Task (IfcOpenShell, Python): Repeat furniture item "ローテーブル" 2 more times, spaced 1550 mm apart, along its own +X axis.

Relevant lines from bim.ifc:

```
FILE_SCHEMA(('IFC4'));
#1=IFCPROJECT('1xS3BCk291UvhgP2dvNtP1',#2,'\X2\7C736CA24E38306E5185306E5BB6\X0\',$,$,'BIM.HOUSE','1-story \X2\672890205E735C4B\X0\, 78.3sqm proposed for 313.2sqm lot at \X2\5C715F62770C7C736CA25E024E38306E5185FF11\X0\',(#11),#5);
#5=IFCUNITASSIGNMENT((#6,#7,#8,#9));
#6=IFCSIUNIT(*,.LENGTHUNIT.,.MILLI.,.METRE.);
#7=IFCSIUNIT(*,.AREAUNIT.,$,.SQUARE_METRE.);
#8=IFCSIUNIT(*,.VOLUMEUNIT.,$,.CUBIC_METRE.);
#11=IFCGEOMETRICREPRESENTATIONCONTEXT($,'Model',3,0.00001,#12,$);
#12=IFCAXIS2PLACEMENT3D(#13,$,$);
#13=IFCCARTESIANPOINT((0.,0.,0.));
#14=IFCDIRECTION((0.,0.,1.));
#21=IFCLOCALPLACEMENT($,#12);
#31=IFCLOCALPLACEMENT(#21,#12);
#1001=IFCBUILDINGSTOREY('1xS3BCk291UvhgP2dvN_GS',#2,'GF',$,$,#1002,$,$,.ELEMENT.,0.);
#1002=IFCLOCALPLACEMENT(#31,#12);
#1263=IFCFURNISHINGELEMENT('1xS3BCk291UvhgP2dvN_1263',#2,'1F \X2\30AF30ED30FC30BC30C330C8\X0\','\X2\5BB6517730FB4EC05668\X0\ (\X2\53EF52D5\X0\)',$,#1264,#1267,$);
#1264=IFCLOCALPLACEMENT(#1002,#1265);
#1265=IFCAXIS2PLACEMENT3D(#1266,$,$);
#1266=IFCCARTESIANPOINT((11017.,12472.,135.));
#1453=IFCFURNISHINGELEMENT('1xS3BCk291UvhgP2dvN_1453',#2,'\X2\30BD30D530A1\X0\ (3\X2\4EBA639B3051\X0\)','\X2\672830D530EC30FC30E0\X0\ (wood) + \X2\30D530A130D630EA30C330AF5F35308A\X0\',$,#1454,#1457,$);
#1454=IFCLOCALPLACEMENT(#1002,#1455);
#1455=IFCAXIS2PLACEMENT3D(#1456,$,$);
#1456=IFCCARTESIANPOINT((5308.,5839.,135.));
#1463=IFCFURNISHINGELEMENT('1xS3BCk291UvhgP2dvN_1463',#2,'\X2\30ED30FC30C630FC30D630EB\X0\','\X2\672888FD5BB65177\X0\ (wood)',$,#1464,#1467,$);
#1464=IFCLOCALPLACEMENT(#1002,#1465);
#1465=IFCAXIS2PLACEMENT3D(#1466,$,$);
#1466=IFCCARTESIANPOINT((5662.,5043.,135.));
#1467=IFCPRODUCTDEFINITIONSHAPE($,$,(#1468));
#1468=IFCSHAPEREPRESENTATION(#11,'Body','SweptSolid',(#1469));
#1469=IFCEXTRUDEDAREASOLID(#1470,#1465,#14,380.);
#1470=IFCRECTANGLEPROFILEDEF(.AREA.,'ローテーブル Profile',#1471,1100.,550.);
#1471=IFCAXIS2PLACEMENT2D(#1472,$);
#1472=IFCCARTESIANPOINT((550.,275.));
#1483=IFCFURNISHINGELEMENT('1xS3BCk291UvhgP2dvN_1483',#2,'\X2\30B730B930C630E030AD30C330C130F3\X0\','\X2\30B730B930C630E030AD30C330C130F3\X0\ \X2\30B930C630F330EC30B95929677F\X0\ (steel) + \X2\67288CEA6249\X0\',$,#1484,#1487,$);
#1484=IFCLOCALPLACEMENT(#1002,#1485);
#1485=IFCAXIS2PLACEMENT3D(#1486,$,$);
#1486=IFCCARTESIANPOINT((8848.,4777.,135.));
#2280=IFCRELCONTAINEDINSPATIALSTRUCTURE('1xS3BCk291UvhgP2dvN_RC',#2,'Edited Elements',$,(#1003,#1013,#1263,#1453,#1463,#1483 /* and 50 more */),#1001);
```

```python
import ifcopenshell
import ifcopenshell.api.geometry
import ifcopenshell.api.root
import ifcopenshell.util.element
import ifcopenshell.util.placement

model = ifcopenshell.open("bim.ifc")


def reuse_history(source, copy):
    """copy_class also copies each property set's owner history, people and application; keep the originals."""
    for rel in copy.IsDefinedBy:
        if rel.is_a("IfcRelDefinesByProperties") and (history := rel.RelatingPropertyDefinition.OwnerHistory):
            rel.RelatingPropertyDefinition.OwnerHistory = source.OwnerHistory
            ifcopenshell.util.element.remove_deep2(model, history)


source = model.by_guid("1xS3BCk291UvhgP2dvN_1463")
base = ifcopenshell.util.placement.get_local_placement(source.ObjectPlacement)
step = base[:3, 0] * 1550.0

for i in range(1, 3):
    copy = ifcopenshell.api.root.copy_class(model, product=source)
    copy.Representation = ifcopenshell.util.element.copy_deep(
        model, source.Representation, exclude=["IfcGeometricRepresentationContext", "IfcRepresentationMap"]
    )
    reuse_history(source, copy)
    matrix = base.copy()
    matrix[:3, 3] += i * step
    print("added at", matrix[:3, 3].round(3) + 0.0)
    ifcopenshell.api.geometry.edit_object_placement(model, product=copy, matrix=matrix, is_si=False)

model.write("bim_v2.ifc")
```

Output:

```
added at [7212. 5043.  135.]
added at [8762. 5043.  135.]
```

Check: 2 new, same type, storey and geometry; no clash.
